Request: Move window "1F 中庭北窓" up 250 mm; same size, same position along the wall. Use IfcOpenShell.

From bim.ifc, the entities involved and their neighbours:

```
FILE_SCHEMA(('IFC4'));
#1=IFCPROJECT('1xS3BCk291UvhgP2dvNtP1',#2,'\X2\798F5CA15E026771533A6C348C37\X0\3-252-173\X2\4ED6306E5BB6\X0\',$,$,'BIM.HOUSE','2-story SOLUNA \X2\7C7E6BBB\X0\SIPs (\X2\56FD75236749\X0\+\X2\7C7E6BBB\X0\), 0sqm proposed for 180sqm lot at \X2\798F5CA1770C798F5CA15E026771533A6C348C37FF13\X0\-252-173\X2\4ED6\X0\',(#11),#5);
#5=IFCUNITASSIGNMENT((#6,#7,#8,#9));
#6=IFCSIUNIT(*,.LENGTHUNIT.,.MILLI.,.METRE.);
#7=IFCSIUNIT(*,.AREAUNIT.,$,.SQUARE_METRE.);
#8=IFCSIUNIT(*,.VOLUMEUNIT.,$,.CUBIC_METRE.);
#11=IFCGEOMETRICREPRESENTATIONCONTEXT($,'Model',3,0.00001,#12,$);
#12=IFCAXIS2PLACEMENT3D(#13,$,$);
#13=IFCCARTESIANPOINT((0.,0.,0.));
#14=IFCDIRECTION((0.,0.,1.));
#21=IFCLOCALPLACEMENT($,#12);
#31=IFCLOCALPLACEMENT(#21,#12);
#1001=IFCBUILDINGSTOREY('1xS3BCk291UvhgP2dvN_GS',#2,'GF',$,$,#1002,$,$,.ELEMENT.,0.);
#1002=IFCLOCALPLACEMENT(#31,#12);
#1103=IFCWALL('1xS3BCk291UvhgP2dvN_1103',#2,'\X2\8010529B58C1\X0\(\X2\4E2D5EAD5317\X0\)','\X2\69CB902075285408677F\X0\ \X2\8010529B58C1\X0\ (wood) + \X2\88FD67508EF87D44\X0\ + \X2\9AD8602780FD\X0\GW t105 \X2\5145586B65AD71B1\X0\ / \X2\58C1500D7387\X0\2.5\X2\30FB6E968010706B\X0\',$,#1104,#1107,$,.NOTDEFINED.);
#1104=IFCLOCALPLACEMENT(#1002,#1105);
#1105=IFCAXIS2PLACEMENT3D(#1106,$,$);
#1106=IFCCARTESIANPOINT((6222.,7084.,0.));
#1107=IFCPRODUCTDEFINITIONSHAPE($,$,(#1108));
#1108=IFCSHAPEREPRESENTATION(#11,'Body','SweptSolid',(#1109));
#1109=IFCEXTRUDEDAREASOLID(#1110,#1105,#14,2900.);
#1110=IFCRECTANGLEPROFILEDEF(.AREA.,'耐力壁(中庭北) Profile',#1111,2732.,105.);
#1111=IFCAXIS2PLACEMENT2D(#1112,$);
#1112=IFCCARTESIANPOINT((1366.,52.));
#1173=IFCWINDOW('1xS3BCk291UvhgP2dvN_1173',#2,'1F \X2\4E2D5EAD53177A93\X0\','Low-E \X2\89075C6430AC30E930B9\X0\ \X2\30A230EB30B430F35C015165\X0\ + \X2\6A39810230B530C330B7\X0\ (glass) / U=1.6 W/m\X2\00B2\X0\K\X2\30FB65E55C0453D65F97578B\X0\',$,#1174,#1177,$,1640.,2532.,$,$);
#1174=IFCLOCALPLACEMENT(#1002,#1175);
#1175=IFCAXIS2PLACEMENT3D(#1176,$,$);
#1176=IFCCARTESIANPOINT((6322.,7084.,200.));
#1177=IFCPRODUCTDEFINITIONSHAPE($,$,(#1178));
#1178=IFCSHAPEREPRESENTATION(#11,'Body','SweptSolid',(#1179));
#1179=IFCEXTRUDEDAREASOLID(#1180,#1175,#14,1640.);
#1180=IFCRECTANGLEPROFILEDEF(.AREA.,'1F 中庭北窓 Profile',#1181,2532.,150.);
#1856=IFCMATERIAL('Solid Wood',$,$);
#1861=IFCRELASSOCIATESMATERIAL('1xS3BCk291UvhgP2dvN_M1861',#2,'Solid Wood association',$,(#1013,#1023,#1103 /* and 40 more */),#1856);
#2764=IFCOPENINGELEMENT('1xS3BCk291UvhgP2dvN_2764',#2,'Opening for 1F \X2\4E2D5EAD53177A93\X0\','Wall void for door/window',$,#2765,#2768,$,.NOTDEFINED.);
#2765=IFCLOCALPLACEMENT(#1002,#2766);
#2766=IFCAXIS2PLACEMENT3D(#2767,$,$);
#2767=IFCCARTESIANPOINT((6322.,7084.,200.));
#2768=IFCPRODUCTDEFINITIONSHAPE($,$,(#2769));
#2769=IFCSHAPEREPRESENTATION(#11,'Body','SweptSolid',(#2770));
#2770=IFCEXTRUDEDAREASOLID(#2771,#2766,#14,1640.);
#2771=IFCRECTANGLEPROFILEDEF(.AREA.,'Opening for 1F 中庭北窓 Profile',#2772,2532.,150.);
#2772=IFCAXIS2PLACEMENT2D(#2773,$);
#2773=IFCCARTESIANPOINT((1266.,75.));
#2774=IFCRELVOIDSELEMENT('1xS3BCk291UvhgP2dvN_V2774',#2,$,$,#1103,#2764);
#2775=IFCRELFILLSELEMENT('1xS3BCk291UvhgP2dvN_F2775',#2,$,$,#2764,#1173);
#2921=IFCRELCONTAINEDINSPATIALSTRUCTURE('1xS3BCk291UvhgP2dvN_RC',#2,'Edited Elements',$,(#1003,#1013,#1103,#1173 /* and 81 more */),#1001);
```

```python
import numpy as np
import ifcopenshell
import ifcopenshell.api.geometry
import ifcopenshell.util.placement
import ifcopenshell.util.unit

model = ifcopenshell.open("bim.ifc")
unit_scale = ifcopenshell.util.unit.calculate_unit_scale(model)

window = model.by_guid("1xS3BCk291UvhgP2dvN_1173")
opening = window.FillsVoids[0].RelatingOpeningElement
dz = 0.25 / unit_scale

shift = np.array([0.0, 0.0, dz])
# The window is not placed relative to its opening, so move both.
for product in (opening, window):
    matrix = ifcopenshell.util.placement.get_local_placement(product.ObjectPlacement)
    matrix[:3, 3] += shift
    ifcopenshell.api.geometry.edit_object_placement(model, product=product, matrix=matrix, is_si=False)

print(f"moved by {dz * unit_scale:+.3f} m")

model.write("bim_edited.ifc")
```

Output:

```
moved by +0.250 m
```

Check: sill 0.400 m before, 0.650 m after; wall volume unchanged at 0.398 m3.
